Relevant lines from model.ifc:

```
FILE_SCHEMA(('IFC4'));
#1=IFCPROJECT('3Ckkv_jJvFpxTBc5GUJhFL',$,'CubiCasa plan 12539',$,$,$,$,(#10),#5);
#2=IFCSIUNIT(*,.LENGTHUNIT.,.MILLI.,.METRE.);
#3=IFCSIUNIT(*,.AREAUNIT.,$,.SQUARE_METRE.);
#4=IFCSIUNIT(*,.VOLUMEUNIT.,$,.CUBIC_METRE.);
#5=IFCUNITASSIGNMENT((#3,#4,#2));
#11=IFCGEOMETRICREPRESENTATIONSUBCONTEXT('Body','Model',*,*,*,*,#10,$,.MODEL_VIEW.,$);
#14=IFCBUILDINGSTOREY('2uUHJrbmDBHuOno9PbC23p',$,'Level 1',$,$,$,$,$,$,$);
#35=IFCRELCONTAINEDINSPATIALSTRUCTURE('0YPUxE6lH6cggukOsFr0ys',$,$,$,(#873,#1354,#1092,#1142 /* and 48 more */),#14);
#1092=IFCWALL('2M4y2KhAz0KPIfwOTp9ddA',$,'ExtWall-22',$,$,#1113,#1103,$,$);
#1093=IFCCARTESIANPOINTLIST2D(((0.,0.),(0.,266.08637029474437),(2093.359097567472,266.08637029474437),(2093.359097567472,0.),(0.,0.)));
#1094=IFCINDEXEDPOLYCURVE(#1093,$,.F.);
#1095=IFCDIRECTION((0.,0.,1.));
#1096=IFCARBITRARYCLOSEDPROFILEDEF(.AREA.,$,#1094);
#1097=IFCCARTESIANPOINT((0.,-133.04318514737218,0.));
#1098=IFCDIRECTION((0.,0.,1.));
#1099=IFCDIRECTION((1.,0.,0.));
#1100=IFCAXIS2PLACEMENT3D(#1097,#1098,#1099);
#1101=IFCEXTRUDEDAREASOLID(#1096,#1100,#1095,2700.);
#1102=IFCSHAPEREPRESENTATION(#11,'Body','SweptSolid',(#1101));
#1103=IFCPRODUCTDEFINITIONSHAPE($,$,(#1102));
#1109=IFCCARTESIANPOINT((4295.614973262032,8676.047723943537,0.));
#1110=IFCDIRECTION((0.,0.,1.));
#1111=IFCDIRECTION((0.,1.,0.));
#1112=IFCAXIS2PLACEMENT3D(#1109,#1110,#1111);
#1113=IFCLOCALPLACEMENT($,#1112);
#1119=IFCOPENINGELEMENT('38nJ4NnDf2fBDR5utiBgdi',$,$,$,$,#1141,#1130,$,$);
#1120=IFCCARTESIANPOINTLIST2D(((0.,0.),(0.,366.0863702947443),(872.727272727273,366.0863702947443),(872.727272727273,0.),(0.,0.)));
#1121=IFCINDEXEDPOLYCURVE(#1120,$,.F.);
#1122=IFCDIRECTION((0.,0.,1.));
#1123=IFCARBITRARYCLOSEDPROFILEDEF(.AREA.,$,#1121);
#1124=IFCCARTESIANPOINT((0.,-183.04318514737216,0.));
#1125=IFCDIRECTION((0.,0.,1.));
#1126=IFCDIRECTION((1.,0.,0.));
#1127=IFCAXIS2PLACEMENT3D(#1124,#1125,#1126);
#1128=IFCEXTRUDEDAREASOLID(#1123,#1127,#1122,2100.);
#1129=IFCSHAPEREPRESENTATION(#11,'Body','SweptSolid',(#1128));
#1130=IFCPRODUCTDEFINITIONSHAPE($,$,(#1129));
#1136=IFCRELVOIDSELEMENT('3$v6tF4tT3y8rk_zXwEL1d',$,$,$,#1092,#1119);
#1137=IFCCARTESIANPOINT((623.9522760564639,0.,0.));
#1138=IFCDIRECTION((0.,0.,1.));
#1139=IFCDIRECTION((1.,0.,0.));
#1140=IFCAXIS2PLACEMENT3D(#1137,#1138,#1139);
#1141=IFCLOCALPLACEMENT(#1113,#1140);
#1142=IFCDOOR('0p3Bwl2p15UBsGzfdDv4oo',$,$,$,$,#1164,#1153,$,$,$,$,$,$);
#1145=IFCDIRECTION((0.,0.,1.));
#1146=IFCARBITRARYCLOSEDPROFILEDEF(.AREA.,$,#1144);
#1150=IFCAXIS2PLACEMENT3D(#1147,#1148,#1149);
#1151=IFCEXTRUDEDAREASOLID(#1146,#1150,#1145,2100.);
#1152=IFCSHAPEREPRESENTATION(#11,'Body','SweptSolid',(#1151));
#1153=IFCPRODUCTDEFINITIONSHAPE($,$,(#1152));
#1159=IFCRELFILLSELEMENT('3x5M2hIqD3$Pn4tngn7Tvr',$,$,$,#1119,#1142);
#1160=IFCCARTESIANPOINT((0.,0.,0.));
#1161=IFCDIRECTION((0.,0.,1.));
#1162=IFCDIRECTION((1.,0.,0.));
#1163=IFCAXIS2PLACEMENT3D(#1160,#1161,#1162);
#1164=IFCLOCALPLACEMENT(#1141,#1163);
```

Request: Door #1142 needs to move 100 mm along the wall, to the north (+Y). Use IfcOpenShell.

```python
import ifcopenshell
import ifcopenshell.api.geometry
import ifcopenshell.util.placement
import ifcopenshell.util.unit

model = ifcopenshell.open("model.ifc")
unit_scale = ifcopenshell.util.unit.calculate_unit_scale(model)

door = model.by_guid("0p3Bwl2p15UBsGzfdDv4oo")
opening = door.FillsVoids[0].RelatingOpeningElement
wall = opening.VoidsElements[0].RelatingBuildingElement

wall_matrix = ifcopenshell.util.placement.get_local_placement(wall.ObjectPlacement)
shift = wall_matrix[:3, 0] * 0.1 / unit_scale
before = ifcopenshell.util.placement.get_local_placement(door.ObjectPlacement)[:3, 3].copy()

# The door is placed relative to its opening, so it follows when the opening moves.
matrix = ifcopenshell.util.placement.get_local_placement(opening.ObjectPlacement)
matrix[:3, 3] += shift
ifcopenshell.api.geometry.edit_object_placement(
    model, product=opening, matrix=matrix, is_si=False, should_transform_children=True
)

after = ifcopenshell.util.placement.get_local_placement(door.ObjectPlacement)[:3, 3]
print("door moved by", (after - before).round(3) + 0.0)

model.write("model_updated.ifc")
```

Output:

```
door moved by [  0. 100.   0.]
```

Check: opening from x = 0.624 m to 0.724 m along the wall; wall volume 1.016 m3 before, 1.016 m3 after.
